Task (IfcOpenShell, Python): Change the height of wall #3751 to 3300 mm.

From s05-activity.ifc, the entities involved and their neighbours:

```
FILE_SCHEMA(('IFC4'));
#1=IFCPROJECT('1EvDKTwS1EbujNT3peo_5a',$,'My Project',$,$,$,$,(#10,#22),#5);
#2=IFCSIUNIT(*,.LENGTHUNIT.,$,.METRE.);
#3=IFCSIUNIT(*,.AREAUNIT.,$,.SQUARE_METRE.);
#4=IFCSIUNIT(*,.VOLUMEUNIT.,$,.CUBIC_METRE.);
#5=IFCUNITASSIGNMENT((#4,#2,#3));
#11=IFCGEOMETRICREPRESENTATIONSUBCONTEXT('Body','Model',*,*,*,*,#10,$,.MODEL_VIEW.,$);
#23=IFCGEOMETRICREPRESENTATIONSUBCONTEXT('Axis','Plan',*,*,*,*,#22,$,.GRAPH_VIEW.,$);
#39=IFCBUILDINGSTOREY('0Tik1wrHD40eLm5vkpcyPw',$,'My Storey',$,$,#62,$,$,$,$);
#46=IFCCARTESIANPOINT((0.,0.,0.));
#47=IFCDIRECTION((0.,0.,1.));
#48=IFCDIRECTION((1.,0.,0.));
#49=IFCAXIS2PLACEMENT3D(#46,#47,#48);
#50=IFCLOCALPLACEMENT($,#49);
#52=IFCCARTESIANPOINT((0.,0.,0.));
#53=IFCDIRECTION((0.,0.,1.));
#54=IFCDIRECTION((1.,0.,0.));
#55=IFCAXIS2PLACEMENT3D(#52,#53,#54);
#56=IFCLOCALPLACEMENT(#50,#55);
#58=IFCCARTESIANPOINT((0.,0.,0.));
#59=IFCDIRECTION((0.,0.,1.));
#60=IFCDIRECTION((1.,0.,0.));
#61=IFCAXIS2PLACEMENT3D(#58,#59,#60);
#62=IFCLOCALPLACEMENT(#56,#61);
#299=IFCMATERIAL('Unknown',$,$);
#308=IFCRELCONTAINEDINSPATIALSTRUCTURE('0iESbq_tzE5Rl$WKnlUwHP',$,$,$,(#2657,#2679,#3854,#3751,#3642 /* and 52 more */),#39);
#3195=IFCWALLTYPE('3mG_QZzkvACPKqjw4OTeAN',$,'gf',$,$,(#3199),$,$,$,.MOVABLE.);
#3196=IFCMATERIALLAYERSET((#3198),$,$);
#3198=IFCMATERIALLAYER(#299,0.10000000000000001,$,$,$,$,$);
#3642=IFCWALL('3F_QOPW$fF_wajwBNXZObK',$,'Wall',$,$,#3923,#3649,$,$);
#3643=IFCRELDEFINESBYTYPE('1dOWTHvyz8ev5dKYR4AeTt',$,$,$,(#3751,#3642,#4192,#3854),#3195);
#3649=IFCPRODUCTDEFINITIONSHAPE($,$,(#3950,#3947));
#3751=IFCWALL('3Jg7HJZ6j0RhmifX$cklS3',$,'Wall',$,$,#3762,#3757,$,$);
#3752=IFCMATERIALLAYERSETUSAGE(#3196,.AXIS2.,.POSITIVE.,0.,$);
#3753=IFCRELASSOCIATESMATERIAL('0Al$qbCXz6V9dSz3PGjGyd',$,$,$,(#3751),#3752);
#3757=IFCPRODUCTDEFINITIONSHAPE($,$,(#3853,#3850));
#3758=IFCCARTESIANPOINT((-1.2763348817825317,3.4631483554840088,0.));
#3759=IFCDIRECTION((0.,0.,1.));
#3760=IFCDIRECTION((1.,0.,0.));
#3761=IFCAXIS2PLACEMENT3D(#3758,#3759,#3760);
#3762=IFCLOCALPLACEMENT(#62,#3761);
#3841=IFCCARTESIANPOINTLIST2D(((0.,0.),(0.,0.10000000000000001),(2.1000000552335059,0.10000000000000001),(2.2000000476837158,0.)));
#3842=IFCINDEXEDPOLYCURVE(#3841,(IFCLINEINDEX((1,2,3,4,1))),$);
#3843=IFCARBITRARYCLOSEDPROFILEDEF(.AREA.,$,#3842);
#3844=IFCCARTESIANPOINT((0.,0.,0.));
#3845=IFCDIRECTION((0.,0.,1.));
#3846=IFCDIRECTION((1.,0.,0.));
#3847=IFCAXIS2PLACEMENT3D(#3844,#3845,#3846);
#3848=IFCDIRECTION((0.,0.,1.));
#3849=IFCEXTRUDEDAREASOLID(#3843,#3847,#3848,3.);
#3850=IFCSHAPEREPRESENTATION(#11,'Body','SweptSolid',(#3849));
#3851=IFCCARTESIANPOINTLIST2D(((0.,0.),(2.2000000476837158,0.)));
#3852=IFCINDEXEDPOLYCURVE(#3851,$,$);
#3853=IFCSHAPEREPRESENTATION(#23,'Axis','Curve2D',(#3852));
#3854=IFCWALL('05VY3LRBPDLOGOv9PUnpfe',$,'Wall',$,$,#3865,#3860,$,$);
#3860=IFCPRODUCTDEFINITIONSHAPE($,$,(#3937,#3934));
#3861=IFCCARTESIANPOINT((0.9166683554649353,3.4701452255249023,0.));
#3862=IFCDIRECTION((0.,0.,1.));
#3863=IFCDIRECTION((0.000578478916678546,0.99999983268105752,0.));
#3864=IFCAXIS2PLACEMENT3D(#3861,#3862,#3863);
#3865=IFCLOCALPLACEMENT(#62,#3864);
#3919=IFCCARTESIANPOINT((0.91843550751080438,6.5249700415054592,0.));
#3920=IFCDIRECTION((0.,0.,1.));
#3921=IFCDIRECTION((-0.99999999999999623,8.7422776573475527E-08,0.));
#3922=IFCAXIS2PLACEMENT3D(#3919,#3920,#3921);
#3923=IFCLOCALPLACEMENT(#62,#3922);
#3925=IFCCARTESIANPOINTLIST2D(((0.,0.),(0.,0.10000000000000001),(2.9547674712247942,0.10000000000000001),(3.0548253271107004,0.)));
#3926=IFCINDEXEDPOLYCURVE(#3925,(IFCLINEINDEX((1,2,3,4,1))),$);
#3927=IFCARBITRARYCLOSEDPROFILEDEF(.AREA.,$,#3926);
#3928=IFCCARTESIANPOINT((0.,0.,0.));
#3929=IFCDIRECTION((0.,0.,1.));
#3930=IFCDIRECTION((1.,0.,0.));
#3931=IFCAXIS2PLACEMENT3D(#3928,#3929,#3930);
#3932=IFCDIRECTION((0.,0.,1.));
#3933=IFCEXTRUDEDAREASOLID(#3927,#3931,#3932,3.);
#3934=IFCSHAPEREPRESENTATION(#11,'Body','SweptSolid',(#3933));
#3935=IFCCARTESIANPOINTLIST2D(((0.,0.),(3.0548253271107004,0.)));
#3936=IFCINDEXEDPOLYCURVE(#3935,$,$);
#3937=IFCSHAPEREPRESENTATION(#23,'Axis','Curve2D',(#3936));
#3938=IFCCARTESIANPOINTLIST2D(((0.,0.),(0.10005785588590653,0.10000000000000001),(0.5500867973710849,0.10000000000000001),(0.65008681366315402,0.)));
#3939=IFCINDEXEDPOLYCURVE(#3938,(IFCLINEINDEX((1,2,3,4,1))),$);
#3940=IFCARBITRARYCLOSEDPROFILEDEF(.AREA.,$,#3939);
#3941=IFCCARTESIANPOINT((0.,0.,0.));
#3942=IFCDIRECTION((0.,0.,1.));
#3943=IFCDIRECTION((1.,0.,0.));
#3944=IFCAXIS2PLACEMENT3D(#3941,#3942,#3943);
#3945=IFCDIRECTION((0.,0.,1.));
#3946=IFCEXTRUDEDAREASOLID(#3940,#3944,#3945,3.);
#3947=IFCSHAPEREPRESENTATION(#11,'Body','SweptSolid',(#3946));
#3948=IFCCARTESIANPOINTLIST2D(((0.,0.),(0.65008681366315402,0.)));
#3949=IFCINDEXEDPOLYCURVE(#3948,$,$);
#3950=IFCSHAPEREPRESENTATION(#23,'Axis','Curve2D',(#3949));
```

```python
import ifcopenshell
import ifcopenshell.geom
import ifcopenshell.util.representation
import ifcopenshell.util.shape
import ifcopenshell.util.unit

model = ifcopenshell.open("s05-activity.ifc")
unit_scale = ifcopenshell.util.unit.calculate_unit_scale(model)
settings = ifcopenshell.geom.settings()


def volume(element):
    """Net volume in cubic metres, openings subtracted."""
    shape = ifcopenshell.geom.create_shape(settings, element)
    return ifcopenshell.util.shape.get_volume(shape.geometry)


wall = model.by_guid("3Jg7HJZ6j0RhmifX$cklS3")
before = volume(wall)

body = ifcopenshell.util.representation.get_representation(wall, "Model", "Body")
solid = body.Items[0]
old_height = solid.Depth
solid.Depth = 3.3 / unit_scale
after = volume(wall)

print(f"height {old_height:g} -> {solid.Depth:g}, volume {before:.3f} -> {after:.3f} m3")

model.write("s05-activity_updated.ifc")
```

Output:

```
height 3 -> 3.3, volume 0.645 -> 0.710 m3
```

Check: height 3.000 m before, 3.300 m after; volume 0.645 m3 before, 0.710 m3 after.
